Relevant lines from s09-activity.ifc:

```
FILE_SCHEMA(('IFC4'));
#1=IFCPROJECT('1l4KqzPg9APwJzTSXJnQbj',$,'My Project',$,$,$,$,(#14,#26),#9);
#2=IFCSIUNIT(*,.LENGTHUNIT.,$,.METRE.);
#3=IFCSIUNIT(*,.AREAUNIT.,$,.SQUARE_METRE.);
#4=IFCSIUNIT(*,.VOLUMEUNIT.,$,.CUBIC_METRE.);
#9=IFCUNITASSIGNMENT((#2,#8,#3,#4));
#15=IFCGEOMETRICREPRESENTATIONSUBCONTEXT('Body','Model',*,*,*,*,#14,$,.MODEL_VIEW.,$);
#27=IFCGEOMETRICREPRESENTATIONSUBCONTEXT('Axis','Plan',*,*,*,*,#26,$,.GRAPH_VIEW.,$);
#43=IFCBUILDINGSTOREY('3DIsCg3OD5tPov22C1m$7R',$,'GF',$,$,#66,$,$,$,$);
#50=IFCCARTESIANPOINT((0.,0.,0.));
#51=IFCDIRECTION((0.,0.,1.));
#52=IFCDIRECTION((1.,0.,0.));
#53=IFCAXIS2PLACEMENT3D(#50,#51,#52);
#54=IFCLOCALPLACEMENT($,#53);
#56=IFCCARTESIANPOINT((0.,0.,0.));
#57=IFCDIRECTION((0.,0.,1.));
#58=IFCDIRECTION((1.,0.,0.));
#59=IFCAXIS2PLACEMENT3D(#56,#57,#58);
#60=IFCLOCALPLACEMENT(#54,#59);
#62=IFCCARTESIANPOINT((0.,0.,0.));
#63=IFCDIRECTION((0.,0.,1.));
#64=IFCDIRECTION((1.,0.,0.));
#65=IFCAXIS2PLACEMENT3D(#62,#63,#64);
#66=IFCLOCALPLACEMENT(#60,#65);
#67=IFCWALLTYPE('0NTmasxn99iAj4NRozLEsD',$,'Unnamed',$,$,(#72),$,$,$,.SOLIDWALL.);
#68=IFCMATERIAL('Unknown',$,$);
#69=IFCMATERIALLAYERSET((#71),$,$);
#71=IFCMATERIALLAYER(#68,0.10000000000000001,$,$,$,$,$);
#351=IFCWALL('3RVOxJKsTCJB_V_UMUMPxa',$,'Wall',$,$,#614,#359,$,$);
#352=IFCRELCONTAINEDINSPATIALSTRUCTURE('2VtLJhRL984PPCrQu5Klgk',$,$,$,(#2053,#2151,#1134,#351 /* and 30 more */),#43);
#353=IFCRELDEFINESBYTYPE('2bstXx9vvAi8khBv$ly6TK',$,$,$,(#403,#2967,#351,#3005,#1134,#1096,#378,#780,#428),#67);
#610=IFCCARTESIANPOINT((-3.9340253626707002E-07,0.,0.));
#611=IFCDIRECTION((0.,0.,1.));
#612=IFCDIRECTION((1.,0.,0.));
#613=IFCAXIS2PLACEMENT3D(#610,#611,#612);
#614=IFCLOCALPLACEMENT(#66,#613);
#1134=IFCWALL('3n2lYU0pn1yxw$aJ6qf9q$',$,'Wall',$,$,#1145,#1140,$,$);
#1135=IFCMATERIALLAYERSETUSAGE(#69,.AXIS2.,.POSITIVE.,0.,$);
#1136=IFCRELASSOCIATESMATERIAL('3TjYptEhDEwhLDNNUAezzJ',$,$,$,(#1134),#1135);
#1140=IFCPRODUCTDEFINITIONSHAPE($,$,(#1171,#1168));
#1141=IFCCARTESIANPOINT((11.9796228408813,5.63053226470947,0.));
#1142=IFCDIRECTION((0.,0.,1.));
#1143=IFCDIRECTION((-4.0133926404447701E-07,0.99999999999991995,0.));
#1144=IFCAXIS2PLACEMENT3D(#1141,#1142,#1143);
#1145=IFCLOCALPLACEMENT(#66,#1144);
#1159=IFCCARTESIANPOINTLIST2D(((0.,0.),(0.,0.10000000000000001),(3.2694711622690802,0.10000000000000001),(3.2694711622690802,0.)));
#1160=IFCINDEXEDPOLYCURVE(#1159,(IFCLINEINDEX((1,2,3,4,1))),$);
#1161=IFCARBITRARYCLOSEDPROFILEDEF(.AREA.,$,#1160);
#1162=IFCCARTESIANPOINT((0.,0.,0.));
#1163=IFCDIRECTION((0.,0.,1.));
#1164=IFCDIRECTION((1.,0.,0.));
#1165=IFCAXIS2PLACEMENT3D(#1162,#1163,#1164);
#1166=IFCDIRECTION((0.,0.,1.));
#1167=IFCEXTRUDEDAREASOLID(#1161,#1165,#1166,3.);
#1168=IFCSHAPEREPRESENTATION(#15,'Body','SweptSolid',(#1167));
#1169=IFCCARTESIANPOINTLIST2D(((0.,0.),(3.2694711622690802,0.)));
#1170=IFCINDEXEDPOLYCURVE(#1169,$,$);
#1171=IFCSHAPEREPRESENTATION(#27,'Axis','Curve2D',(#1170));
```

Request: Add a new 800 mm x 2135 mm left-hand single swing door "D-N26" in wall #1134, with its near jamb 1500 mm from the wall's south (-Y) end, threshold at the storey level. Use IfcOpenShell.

```python
import numpy as np
import ifcopenshell
import ifcopenshell.api.feature
import ifcopenshell.api.geometry
import ifcopenshell.api.root
import ifcopenshell.api.spatial
import ifcopenshell.geom
import ifcopenshell.util.element
import ifcopenshell.util.placement
import ifcopenshell.util.representation
import ifcopenshell.util.shape
import ifcopenshell.util.unit

model = ifcopenshell.open("s09-activity.ifc")
unit_scale = ifcopenshell.util.unit.calculate_unit_scale(model)
settings = ifcopenshell.geom.settings()


def volume(element):
    """Net volume in cubic metres, openings subtracted."""
    shape = ifcopenshell.geom.create_shape(settings, element)
    return ifcopenshell.util.shape.get_volume(shape.geometry)


wall = model.by_guid("3n2lYU0pn1yxw$aJ6qf9q$")
storey = ifcopenshell.util.element.get_container(wall, ifc_class="IfcBuildingStorey")
context = ifcopenshell.util.representation.get_context(model, "Model", "Body", "MODEL_VIEW")
before = volume(wall)

width, height, from_end, sill = 0.8, 2.135, 1.5, 0.0  # metres

# The wall runs along its own X axis, and the end named is its -X end.
wall_shape = ifcopenshell.geom.create_shape(settings, wall)
x, y, z = ifcopenshell.util.shape.get_vertices(wall_shape.geometry).T
start = x.min() + from_end
face, thickness = float(y.min()), float(y.max() - y.min())
wall_matrix = ifcopenshell.util.placement.get_local_placement(wall.ObjectPlacement)
level = ifcopenshell.util.placement.get_local_placement(storey.ObjectPlacement)[2, 3]


def in_wall(x, y):
    """Placement at x, y metres in the wall's axes, at sill height."""
    matrix = wall_matrix.copy()
    matrix[:, 3] = wall_matrix @ np.array([x / unit_scale, y / unit_scale, 0.0, 1.0])
    matrix[2, 3] = level + sill / unit_scale
    return matrix


# Opening: a box that overshoots both wall faces by 50 mm.
opening = ifcopenshell.api.root.create_entity(model, ifc_class="IfcOpeningElement", predefined_type="OPENING")
box = ifcopenshell.api.geometry.add_wall_representation(
    model, context=context, length=width, height=height, thickness=thickness + 0.1
)
ifcopenshell.api.geometry.assign_representation(model, product=opening, representation=box)
ifcopenshell.api.geometry.edit_object_placement(model, product=opening, matrix=in_wall(start, face - 0.05), is_si=False)
ifcopenshell.api.feature.add_feature(model, feature=opening, element=wall)

door = ifcopenshell.api.root.create_entity(model, ifc_class="IfcDoor", name="D-N26", predefined_type="DOOR")
door.OverallWidth, door.OverallHeight = width / unit_scale, height / unit_scale
door.OperationType = "SINGLE_SWING_LEFT"
body = ifcopenshell.api.geometry.add_door_representation(
    model,
    context=context,
    overall_width=door.OverallWidth,
    overall_height=door.OverallHeight,
    operation_type="SINGLE_SWING_LEFT",
    lining_properties={"LiningDepth": thickness / unit_scale, "ThresholdDepth": thickness / unit_scale},
)
ifcopenshell.api.geometry.assign_representation(model, product=door, representation=body)
ifcopenshell.api.spatial.assign_container(model, products=[door], relating_structure=storey)
ifcopenshell.api.feature.add_filling(model, opening=opening, element=door)

# The lining spans the wall, so the door starts at the wall face.
ifcopenshell.api.geometry.edit_object_placement(model, product=door, matrix=in_wall(start, face), is_si=False)

after = volume(wall)

print(f"wall volume {before:.3f} -> {after:.3f} m3")

model.write("s09-activity-out.ifc")
```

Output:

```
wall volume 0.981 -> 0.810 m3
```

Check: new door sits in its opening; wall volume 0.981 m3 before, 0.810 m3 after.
